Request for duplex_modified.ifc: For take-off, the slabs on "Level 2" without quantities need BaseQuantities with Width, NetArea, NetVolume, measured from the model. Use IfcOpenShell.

First a look at what the model holds.

```python
import ifcopenshell
import ifcopenshell.util.element
import ifcopenshell.util.unit

model = ifcopenshell.open("duplex_modified.ifc")
print(model.schema)
for unit_type in ("LENGTHUNIT", "AREAUNIT", "VOLUMEUNIT"):
    print(unit_type, ifcopenshell.util.unit.calculate_unit_scale(model, unit_type))
storey = next(s for s in model.by_type("IfcBuildingStorey") if s.Name == "Level 2")
slabs = [e for e in ifcopenshell.util.element.get_decomposition(storey) if e.is_a("IfcSlab")]
for e in sorted(slabs, key=lambda e: e.id()):
    print(e.id(), e.is_a(), e.Name, list(ifcopenshell.util.element.get_psets(e, qtos_only=True)), sep=" | ")
```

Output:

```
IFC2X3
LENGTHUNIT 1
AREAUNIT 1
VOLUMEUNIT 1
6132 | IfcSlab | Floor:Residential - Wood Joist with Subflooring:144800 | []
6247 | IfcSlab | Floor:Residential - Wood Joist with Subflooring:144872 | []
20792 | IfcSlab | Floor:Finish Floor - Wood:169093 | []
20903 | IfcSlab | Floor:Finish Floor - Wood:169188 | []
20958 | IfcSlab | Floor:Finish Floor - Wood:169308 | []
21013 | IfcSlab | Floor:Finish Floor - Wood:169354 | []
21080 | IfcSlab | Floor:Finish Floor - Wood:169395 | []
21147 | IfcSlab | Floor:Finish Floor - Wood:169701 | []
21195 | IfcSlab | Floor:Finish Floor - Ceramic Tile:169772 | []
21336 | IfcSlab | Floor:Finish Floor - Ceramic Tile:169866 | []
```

```python
import ifcopenshell
import ifcopenshell.api.pset
import ifcopenshell.geom
import ifcopenshell.util.element
import ifcopenshell.util.shape
import ifcopenshell.util.unit

model = ifcopenshell.open("duplex_modified.ifc")
unit_scale = ifcopenshell.util.unit.calculate_unit_scale(model)
area_scale = ifcopenshell.util.unit.calculate_unit_scale(model, "AREAUNIT")
volume_scale = ifcopenshell.util.unit.calculate_unit_scale(model, "VOLUMEUNIT")
settings = ifcopenshell.geom.settings()

storey = next(s for s in model.by_type("IfcBuildingStorey") if s.Name == "Level 2")
slabs = [e for e in ifcopenshell.util.element.get_decomposition(storey) if e.is_a("IfcSlab")]

for e in sorted(slabs, key=lambda e: e.id()):
    if ifcopenshell.util.element.get_psets(e, qtos_only=True, should_inherit=False):
        continue
    # Geometry comes back in metres, in the element's own axes.
    shape = ifcopenshell.geom.create_shape(settings, e)
    values = {
        "Width": ifcopenshell.util.shape.get_z(shape.geometry) / unit_scale,
        "NetArea": ifcopenshell.util.shape.get_footprint_area(shape.geometry) / area_scale,
        "NetVolume": ifcopenshell.util.shape.get_volume(shape.geometry) / volume_scale,
    }
    qto = ifcopenshell.api.pset.add_qto(model, product=e, name="BaseQuantities")
    ifcopenshell.api.pset.edit_qto(model, qto=qto, properties=values)
    print(e.id(), {k: round(v, 3) for k, v in values.items()})

model.write("duplex_modified_edited.ifc")
```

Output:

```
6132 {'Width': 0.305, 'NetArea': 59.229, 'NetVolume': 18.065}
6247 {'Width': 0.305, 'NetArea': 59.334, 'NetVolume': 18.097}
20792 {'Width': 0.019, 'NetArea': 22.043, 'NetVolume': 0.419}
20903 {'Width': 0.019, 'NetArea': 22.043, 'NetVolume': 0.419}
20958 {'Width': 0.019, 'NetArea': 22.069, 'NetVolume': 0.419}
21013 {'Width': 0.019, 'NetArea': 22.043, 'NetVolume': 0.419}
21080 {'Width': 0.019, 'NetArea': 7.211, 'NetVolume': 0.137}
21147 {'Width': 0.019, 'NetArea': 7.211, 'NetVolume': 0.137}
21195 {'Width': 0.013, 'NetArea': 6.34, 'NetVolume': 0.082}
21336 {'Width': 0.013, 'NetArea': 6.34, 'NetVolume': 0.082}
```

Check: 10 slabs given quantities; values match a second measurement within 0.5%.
